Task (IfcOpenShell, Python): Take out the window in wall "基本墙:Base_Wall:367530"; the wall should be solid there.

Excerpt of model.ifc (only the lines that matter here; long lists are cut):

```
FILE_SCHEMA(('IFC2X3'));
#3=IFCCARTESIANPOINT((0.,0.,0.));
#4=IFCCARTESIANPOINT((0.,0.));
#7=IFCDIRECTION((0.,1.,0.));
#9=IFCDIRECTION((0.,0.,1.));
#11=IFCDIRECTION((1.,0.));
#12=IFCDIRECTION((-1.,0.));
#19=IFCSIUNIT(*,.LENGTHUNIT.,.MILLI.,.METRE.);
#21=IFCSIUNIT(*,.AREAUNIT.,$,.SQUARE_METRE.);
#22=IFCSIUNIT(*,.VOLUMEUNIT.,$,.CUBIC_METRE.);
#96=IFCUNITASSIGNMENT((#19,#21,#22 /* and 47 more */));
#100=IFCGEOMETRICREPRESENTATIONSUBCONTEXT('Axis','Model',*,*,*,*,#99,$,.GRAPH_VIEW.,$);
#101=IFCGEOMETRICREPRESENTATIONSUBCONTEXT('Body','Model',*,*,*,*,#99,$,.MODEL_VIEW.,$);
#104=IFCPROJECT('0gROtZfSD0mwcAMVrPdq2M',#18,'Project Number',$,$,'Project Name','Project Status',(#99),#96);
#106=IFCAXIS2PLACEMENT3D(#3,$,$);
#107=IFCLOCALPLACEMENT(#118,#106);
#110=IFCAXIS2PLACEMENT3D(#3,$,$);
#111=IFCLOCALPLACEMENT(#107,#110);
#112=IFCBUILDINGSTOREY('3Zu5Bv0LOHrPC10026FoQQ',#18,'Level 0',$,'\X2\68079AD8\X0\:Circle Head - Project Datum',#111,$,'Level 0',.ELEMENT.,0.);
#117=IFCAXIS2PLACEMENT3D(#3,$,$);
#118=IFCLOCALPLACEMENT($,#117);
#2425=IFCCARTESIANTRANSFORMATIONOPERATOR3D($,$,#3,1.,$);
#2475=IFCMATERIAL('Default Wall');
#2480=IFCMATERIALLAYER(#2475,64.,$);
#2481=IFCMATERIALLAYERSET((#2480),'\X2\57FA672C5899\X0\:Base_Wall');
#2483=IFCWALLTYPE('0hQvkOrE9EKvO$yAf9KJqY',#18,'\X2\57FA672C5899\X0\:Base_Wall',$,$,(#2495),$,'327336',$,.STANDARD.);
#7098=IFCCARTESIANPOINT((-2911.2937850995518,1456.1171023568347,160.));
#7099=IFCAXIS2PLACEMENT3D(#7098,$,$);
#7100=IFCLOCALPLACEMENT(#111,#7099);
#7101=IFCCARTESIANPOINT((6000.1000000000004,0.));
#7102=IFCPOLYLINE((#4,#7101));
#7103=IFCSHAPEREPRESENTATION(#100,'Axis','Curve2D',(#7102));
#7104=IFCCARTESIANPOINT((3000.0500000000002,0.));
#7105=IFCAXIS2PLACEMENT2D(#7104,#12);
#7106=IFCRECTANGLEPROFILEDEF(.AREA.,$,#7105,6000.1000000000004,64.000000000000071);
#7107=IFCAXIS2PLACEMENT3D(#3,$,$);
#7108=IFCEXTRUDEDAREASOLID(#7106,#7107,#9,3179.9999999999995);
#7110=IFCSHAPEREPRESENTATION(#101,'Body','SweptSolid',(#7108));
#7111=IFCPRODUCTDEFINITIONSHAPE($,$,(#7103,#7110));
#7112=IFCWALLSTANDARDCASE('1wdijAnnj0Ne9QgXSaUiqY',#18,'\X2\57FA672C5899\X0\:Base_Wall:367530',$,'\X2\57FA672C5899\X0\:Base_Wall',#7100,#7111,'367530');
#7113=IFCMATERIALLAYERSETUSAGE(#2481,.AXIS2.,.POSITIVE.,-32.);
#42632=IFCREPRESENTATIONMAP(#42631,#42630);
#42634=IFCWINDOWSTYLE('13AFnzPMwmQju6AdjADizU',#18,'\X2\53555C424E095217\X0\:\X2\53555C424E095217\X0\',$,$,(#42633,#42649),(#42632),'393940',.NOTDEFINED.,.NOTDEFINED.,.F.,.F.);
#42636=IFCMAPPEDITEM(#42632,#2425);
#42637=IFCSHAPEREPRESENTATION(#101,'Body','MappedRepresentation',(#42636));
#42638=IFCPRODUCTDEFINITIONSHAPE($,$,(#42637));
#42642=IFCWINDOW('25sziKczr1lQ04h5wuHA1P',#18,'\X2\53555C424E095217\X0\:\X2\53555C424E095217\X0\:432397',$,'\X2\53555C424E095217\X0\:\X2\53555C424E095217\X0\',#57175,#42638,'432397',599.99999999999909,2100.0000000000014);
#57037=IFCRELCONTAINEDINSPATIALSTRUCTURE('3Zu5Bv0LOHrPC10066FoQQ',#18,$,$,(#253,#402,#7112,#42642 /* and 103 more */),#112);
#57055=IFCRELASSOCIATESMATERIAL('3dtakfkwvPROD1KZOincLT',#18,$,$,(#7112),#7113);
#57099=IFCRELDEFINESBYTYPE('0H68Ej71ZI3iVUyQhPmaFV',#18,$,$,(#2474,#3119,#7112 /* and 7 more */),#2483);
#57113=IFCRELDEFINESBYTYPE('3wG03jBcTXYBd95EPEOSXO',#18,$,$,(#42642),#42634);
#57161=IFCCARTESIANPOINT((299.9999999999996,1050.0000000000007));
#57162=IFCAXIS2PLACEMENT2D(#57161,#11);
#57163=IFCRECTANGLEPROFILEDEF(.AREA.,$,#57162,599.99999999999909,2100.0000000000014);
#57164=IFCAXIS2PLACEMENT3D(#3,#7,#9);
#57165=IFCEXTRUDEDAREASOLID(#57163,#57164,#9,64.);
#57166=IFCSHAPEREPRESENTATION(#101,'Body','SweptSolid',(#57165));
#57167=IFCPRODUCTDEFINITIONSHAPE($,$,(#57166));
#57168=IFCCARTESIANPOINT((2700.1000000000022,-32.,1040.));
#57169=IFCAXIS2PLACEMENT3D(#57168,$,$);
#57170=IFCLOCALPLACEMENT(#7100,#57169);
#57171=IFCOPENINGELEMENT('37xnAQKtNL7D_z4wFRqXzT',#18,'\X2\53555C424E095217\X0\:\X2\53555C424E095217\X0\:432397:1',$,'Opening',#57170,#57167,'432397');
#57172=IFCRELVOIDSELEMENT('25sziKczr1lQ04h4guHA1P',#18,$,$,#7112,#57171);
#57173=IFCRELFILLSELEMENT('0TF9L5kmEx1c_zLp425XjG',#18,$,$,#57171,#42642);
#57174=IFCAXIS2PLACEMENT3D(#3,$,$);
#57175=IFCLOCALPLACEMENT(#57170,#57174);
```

```python
import ifcopenshell
import ifcopenshell.api.feature
import ifcopenshell.api.root
import ifcopenshell.geom
import ifcopenshell.util.shape

model = ifcopenshell.open("model.ifc")
settings = ifcopenshell.geom.settings()


def volume(element):
    """Net volume in cubic metres, openings subtracted."""
    shape = ifcopenshell.geom.create_shape(settings, element)
    return ifcopenshell.util.shape.get_volume(shape.geometry)


window = model.by_id(42642)
opening = window.FillsVoids[0].RelatingOpeningElement
wall = opening.VoidsElements[0].RelatingBuildingElement
before = volume(wall)

ifcopenshell.api.root.remove_product(model, product=window)
ifcopenshell.api.feature.remove_feature(model, feature=opening)

after = volume(wall)

print(f"wall volume {before:.3f} -> {after:.3f} m3")

model.write("model_edited.ifc")
```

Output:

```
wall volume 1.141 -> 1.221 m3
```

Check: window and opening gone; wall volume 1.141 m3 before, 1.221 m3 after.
